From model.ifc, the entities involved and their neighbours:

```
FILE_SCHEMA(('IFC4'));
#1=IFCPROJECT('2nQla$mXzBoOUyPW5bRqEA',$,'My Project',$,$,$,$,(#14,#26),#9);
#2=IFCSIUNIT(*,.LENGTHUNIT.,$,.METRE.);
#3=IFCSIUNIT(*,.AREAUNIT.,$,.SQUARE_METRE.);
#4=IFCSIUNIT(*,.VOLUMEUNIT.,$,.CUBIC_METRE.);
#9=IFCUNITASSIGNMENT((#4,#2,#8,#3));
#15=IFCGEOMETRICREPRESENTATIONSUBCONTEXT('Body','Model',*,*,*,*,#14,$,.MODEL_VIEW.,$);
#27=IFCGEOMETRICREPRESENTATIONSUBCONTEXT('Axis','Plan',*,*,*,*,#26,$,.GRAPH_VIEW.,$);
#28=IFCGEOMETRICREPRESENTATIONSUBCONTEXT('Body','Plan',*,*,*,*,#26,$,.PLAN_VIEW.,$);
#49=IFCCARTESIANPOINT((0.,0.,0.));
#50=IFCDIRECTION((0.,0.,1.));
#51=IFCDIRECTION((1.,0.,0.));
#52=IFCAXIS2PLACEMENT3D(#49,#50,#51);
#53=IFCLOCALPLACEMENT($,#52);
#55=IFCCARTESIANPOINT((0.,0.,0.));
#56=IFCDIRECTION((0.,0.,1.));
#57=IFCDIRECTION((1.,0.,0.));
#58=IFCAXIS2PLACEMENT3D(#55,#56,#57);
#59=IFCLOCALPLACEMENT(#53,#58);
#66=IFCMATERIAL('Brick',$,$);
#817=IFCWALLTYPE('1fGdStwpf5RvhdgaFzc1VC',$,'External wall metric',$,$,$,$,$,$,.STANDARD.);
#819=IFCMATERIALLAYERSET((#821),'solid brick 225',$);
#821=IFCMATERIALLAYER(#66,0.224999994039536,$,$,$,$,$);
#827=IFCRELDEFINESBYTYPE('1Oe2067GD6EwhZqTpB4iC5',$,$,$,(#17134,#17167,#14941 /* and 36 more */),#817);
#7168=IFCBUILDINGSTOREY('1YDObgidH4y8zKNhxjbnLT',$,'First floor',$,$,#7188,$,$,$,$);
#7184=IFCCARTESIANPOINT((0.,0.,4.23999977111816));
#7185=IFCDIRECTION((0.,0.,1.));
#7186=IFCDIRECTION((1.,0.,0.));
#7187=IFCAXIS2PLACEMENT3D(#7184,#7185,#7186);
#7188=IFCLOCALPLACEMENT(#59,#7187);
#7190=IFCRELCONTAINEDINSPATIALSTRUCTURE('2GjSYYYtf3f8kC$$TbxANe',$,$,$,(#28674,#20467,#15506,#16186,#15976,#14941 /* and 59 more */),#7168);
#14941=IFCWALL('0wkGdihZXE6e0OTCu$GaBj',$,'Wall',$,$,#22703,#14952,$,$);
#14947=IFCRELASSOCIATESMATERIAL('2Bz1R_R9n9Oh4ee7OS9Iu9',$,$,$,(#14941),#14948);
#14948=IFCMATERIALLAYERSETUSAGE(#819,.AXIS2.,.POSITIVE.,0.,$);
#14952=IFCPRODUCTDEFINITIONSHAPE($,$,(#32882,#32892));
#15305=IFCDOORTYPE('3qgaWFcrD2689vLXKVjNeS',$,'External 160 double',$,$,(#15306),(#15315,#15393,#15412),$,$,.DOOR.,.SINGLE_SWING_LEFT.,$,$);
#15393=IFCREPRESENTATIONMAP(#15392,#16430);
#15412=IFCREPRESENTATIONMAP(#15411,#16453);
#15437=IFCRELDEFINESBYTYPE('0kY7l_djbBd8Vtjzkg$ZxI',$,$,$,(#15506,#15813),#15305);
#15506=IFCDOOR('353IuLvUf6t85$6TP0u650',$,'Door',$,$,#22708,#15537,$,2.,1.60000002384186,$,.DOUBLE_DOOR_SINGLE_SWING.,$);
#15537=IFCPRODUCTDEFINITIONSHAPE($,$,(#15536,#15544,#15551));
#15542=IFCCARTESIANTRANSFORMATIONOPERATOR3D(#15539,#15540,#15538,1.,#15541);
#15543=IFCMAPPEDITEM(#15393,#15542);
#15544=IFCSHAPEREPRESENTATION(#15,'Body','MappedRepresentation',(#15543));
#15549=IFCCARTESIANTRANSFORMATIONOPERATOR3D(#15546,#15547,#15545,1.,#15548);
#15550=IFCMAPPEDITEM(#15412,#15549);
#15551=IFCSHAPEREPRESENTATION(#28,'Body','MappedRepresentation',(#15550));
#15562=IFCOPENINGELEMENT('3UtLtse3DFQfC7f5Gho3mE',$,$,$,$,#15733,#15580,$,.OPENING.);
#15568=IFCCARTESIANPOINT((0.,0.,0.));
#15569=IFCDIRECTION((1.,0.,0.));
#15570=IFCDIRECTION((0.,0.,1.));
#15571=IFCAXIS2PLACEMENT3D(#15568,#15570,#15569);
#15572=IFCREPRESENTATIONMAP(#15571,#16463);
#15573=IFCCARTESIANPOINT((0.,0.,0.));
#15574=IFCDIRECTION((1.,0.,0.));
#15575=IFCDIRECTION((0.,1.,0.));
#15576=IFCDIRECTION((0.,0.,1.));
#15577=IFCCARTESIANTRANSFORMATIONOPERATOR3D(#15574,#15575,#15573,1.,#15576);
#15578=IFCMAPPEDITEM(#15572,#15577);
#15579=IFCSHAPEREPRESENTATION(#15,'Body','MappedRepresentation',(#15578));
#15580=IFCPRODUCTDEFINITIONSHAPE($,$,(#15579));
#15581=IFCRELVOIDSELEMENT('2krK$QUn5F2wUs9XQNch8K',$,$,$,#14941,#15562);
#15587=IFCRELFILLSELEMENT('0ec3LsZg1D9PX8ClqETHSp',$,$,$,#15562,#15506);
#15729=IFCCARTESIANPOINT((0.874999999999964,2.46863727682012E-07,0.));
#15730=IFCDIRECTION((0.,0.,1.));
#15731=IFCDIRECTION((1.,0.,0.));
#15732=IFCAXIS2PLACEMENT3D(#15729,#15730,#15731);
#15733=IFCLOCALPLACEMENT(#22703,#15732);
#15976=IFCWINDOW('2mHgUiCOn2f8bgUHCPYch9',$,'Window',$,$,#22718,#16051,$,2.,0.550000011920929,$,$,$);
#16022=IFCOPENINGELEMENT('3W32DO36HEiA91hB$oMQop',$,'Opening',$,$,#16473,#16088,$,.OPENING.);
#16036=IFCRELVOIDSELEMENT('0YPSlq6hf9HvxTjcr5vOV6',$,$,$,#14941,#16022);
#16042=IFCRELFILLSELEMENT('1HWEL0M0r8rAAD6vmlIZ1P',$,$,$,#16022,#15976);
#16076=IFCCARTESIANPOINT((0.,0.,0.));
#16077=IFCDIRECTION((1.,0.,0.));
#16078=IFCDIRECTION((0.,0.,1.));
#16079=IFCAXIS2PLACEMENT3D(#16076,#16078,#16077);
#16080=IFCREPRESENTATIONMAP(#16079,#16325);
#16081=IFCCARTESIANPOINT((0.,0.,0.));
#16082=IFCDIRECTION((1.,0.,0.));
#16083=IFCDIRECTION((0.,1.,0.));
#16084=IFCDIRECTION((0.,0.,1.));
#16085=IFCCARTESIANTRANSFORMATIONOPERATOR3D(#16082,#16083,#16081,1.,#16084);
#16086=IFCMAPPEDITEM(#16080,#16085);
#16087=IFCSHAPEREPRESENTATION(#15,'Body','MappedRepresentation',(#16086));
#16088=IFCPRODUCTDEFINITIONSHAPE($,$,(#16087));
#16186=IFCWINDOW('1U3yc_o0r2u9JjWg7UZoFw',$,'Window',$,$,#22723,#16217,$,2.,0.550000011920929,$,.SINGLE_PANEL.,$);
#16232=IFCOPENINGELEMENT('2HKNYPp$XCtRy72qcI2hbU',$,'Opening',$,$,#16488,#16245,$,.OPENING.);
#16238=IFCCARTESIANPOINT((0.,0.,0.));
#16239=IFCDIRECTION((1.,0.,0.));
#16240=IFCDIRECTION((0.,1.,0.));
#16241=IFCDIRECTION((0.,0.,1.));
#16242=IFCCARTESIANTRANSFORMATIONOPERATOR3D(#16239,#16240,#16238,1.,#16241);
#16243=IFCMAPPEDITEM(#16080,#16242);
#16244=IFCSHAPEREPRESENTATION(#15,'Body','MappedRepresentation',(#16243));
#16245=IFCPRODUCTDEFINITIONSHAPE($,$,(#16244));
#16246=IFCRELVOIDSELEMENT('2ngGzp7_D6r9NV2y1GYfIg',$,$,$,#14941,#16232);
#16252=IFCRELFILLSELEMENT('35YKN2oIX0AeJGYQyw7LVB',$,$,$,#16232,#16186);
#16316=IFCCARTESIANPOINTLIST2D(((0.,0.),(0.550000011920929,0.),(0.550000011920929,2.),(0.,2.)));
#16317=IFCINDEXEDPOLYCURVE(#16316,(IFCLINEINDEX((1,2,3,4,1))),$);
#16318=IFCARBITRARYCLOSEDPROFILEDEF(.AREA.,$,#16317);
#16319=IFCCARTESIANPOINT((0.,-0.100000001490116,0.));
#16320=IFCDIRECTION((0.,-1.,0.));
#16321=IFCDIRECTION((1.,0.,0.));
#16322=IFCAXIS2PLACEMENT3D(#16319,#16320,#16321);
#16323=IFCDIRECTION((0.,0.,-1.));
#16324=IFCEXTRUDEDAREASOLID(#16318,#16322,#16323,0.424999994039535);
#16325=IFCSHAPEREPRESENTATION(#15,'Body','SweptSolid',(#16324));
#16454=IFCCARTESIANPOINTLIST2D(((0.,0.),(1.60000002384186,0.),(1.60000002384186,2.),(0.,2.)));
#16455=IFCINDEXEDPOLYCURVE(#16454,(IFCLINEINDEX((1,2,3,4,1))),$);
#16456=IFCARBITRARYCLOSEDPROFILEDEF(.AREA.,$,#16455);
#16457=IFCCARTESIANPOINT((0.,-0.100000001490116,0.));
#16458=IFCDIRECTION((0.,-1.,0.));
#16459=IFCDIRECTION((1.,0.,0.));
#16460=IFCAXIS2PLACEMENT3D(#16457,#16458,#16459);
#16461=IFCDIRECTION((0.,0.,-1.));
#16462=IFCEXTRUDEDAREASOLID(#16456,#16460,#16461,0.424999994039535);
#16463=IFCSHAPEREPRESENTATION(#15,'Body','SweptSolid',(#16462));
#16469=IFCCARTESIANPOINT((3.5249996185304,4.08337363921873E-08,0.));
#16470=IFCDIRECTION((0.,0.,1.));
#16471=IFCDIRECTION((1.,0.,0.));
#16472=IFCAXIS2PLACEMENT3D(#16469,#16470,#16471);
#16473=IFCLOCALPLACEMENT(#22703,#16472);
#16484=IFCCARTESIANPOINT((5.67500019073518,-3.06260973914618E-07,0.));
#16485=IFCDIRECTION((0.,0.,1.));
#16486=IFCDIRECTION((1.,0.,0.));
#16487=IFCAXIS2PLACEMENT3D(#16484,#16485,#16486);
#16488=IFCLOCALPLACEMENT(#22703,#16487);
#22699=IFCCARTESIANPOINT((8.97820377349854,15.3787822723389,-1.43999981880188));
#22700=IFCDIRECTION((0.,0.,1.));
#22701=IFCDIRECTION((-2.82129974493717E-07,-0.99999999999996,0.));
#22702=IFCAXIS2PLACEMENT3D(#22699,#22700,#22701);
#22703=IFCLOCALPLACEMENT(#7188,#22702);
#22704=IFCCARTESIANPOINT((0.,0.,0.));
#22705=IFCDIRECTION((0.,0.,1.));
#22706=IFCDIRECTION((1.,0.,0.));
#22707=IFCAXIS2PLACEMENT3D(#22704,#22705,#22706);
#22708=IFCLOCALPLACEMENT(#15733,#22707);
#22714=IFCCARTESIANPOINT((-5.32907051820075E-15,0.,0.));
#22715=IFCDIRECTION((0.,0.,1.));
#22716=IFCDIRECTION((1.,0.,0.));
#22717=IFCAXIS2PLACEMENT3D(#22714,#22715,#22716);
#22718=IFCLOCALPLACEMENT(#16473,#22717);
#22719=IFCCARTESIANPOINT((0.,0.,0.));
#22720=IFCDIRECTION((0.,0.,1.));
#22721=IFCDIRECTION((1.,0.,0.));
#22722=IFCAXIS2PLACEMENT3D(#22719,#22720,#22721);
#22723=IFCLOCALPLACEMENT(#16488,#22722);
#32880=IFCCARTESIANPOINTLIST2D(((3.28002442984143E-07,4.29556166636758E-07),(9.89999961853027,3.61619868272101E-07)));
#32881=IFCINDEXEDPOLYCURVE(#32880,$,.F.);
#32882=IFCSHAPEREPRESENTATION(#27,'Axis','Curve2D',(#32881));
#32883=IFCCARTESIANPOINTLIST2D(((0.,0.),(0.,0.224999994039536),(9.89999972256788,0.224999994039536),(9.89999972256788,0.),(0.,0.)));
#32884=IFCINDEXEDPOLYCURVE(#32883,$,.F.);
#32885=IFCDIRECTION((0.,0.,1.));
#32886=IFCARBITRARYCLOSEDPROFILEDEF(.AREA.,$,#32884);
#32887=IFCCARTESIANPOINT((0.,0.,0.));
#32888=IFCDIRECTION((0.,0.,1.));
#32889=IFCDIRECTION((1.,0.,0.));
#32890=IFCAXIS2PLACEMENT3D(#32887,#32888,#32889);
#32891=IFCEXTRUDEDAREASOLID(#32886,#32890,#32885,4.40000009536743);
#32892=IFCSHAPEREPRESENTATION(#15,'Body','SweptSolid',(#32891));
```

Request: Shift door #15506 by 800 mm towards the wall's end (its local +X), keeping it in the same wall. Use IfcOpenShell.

```python
import ifcopenshell
import ifcopenshell.api.geometry
import ifcopenshell.util.placement

model = ifcopenshell.open("model.ifc")

door = model.by_guid("353IuLvUf6t85$6TP0u650")
opening = door.FillsVoids[0].RelatingOpeningElement
wall = opening.VoidsElements[0].RelatingBuildingElement

wall_matrix = ifcopenshell.util.placement.get_local_placement(wall.ObjectPlacement)
shift = wall_matrix[:3, 0] * 0.8
before = ifcopenshell.util.placement.get_local_placement(door.ObjectPlacement)[:3, 3].copy()

# The door is placed relative to its opening, so it follows when the opening moves.
matrix = ifcopenshell.util.placement.get_local_placement(opening.ObjectPlacement)
matrix[:3, 3] += shift
ifcopenshell.api.geometry.edit_object_placement(
    model, product=opening, matrix=matrix, is_si=False, should_transform_children=True
)

after = ifcopenshell.util.placement.get_local_placement(door.ObjectPlacement)[:3, 3]
print("door moved by", (after - before).round(3) + 0.0)

model.write("model_edited.ifc")
```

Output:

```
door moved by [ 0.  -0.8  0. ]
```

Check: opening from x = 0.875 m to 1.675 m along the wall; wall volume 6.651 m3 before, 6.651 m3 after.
